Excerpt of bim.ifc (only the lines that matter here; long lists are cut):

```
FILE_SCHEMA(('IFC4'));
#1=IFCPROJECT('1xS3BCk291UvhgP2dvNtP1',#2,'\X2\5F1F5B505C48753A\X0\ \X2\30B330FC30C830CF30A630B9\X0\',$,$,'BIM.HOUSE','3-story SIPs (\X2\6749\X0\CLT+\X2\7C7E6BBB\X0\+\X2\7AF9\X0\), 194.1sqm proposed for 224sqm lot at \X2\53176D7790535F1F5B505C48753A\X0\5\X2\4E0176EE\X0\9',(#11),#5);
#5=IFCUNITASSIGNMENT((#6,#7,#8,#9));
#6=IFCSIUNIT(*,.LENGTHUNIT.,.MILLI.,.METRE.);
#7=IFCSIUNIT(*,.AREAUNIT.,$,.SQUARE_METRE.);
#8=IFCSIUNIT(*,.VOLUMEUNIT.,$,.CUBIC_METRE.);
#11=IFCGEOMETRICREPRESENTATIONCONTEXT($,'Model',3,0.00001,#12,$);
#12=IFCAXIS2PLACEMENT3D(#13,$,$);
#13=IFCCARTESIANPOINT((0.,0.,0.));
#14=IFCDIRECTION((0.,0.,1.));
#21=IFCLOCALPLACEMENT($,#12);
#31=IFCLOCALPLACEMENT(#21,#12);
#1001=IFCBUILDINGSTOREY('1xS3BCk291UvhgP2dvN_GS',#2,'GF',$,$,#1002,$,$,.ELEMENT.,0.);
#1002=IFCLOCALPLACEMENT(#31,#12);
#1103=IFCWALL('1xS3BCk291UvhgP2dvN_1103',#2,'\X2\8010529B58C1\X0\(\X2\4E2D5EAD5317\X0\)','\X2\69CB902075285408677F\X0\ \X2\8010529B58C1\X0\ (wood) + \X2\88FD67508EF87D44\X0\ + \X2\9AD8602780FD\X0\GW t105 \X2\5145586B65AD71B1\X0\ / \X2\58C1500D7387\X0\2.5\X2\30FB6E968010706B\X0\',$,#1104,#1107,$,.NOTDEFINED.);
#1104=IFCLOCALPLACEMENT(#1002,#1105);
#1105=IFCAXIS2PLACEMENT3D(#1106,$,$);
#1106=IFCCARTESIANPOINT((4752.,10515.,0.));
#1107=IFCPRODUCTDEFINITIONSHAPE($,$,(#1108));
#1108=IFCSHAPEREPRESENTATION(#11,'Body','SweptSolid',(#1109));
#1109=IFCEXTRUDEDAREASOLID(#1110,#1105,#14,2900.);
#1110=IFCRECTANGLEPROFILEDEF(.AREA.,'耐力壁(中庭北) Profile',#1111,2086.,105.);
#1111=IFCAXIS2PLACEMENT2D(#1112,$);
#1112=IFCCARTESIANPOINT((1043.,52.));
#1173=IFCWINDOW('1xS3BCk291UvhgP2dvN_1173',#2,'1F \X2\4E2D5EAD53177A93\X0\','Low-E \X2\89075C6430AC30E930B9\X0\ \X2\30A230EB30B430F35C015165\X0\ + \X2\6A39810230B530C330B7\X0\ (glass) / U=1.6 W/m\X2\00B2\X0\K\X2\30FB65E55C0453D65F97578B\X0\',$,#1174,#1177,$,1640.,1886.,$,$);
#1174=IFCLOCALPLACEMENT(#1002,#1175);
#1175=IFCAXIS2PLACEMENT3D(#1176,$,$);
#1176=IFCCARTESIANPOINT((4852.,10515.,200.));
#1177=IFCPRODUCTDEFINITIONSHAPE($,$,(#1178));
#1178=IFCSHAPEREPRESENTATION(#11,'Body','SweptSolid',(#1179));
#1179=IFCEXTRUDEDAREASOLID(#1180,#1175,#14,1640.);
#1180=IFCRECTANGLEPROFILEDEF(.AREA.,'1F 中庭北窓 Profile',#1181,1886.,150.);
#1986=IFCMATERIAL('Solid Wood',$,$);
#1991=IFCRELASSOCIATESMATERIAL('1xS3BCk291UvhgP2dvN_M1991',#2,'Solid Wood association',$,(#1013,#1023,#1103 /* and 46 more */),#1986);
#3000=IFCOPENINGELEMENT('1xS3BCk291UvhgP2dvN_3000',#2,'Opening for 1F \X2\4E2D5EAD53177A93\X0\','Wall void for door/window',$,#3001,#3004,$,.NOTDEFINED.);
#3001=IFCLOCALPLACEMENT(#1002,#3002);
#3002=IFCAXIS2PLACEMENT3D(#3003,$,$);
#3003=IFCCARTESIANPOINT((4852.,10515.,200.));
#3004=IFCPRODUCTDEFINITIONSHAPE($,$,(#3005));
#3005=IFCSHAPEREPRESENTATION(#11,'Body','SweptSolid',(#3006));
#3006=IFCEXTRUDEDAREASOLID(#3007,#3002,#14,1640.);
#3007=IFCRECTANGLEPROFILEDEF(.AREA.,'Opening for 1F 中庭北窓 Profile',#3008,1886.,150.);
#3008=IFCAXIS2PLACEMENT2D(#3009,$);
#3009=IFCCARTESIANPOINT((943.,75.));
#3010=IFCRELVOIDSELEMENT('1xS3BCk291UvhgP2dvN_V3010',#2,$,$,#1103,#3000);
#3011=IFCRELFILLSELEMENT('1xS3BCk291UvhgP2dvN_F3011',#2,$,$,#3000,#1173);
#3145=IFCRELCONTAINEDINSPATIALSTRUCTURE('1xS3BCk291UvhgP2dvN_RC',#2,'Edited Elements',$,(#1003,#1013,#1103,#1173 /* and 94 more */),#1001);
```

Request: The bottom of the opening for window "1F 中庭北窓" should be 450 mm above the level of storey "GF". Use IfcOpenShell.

```python
import numpy as np
import ifcopenshell
import ifcopenshell.api.geometry
import ifcopenshell.geom
import ifcopenshell.util.element
import ifcopenshell.util.placement
import ifcopenshell.util.shape
import ifcopenshell.util.unit

model = ifcopenshell.open("bim.ifc")
unit_scale = ifcopenshell.util.unit.calculate_unit_scale(model)

window = model.by_guid("1xS3BCk291UvhgP2dvN_1173")
opening = window.FillsVoids[0].RelatingOpeningElement
storey = ifcopenshell.util.element.get_container(window, ifc_class="IfcBuildingStorey")
level = ifcopenshell.util.placement.get_local_placement(storey.ObjectPlacement)[2, 3]

# The opening's origin need not be at the sill, so measure its lowest point.
shape = ifcopenshell.geom.create_shape(ifcopenshell.geom.settings(), opening)
bottom = ifcopenshell.util.shape.get_shape_bottom_elevation(shape, shape.geometry) / unit_scale
dz = level + 450.0 - bottom

shift = np.array([0.0, 0.0, dz])
# The window is not placed relative to its opening, so move both.
for product in (opening, window):
    matrix = ifcopenshell.util.placement.get_local_placement(product.ObjectPlacement)
    matrix[:3, 3] += shift
    ifcopenshell.api.geometry.edit_object_placement(model, product=product, matrix=matrix, is_si=False)

print(f"moved by {dz * unit_scale:+.3f} m")

model.write("bim_v2.ifc")
```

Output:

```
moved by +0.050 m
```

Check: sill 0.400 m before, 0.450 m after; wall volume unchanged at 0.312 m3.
